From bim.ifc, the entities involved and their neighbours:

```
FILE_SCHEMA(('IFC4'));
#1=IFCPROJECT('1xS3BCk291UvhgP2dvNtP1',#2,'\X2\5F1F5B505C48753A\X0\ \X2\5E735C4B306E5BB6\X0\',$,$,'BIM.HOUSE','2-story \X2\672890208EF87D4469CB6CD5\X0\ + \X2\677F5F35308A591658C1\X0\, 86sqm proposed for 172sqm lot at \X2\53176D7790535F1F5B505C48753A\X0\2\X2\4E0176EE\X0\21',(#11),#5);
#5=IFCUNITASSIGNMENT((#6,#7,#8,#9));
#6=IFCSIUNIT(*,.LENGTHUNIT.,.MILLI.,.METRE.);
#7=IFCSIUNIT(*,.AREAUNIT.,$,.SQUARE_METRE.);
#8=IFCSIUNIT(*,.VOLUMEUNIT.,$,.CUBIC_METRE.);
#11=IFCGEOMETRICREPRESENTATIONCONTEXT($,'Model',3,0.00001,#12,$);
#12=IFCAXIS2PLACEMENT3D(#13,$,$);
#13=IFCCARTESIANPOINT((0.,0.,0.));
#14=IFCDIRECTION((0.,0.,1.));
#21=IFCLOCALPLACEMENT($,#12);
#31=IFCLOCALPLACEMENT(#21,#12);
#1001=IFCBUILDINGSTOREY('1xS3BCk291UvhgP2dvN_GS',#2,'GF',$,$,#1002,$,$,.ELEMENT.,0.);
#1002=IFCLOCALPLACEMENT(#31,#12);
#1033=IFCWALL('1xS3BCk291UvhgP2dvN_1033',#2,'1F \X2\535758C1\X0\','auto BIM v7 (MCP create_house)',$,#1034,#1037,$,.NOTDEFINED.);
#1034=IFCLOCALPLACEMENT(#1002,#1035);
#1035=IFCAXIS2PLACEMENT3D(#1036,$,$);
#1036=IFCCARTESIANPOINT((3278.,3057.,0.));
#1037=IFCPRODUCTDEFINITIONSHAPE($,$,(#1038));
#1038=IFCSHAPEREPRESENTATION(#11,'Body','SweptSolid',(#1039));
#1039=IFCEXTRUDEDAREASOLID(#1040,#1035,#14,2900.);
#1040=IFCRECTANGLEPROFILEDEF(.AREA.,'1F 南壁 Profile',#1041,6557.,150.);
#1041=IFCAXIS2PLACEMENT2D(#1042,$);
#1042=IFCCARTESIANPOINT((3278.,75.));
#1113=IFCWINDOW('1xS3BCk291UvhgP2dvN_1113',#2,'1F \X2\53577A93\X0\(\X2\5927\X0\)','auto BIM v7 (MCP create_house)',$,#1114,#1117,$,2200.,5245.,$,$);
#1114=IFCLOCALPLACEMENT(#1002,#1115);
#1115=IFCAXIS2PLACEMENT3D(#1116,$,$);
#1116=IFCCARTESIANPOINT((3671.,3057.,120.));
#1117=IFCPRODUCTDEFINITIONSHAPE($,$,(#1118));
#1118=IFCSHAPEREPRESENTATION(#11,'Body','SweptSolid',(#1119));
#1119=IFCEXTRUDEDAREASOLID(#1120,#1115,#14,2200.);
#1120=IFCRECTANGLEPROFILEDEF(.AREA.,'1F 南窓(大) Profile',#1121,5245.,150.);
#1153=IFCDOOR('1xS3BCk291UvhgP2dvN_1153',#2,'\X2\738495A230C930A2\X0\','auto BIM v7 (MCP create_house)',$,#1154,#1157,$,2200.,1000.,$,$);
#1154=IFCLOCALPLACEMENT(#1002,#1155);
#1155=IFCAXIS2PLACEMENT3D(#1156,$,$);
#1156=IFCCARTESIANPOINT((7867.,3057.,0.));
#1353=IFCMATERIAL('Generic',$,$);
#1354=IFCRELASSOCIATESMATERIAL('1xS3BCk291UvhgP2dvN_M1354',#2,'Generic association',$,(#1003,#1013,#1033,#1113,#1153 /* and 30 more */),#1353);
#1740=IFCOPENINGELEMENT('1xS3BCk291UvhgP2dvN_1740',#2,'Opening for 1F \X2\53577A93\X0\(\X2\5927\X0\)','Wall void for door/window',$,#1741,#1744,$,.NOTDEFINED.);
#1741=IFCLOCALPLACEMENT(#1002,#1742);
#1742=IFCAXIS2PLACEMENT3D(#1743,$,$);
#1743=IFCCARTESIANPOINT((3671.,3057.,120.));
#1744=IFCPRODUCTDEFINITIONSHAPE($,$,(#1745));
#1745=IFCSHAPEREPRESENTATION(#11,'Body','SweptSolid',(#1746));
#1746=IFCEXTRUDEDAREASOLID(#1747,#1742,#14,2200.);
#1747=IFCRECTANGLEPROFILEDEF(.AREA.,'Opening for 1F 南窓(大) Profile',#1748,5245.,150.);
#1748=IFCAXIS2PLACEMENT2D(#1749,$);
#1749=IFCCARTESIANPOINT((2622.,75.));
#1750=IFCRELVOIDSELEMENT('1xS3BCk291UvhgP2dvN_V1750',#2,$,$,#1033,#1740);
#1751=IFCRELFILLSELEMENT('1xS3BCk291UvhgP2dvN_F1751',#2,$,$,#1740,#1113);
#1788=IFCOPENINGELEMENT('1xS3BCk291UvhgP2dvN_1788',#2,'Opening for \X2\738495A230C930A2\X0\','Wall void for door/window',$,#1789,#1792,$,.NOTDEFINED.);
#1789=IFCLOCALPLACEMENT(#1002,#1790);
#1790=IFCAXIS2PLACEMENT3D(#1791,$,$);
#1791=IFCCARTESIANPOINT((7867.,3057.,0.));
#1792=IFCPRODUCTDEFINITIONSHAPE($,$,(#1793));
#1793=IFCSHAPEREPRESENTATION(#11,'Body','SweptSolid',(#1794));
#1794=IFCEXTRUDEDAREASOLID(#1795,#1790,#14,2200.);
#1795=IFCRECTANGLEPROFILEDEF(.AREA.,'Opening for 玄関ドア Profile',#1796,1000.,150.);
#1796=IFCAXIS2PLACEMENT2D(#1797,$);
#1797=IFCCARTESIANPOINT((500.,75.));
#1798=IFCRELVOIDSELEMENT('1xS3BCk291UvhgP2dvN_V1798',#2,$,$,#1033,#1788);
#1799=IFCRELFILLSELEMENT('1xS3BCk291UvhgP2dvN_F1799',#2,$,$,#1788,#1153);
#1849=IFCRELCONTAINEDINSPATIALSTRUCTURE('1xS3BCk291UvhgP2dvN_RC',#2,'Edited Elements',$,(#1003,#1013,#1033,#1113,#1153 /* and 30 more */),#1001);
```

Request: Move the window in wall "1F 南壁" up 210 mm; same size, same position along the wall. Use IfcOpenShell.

```python
import numpy as np
import ifcopenshell
import ifcopenshell.api.geometry
import ifcopenshell.util.placement
import ifcopenshell.util.unit

model = ifcopenshell.open("bim.ifc")
unit_scale = ifcopenshell.util.unit.calculate_unit_scale(model)

window = model.by_guid("1xS3BCk291UvhgP2dvN_1113")
opening = window.FillsVoids[0].RelatingOpeningElement
dz = 210.0

shift = np.array([0.0, 0.0, dz])
# The window is not placed relative to its opening, so move both.
for product in (opening, window):
    matrix = ifcopenshell.util.placement.get_local_placement(product.ObjectPlacement)
    matrix[:3, 3] += shift
    ifcopenshell.api.geometry.edit_object_placement(model, product=product, matrix=matrix, is_si=False)

print(f"moved by {dz * unit_scale:+.3f} m")

model.write("bim_updated.ifc")
```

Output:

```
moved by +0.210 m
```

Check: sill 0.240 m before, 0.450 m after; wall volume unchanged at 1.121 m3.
